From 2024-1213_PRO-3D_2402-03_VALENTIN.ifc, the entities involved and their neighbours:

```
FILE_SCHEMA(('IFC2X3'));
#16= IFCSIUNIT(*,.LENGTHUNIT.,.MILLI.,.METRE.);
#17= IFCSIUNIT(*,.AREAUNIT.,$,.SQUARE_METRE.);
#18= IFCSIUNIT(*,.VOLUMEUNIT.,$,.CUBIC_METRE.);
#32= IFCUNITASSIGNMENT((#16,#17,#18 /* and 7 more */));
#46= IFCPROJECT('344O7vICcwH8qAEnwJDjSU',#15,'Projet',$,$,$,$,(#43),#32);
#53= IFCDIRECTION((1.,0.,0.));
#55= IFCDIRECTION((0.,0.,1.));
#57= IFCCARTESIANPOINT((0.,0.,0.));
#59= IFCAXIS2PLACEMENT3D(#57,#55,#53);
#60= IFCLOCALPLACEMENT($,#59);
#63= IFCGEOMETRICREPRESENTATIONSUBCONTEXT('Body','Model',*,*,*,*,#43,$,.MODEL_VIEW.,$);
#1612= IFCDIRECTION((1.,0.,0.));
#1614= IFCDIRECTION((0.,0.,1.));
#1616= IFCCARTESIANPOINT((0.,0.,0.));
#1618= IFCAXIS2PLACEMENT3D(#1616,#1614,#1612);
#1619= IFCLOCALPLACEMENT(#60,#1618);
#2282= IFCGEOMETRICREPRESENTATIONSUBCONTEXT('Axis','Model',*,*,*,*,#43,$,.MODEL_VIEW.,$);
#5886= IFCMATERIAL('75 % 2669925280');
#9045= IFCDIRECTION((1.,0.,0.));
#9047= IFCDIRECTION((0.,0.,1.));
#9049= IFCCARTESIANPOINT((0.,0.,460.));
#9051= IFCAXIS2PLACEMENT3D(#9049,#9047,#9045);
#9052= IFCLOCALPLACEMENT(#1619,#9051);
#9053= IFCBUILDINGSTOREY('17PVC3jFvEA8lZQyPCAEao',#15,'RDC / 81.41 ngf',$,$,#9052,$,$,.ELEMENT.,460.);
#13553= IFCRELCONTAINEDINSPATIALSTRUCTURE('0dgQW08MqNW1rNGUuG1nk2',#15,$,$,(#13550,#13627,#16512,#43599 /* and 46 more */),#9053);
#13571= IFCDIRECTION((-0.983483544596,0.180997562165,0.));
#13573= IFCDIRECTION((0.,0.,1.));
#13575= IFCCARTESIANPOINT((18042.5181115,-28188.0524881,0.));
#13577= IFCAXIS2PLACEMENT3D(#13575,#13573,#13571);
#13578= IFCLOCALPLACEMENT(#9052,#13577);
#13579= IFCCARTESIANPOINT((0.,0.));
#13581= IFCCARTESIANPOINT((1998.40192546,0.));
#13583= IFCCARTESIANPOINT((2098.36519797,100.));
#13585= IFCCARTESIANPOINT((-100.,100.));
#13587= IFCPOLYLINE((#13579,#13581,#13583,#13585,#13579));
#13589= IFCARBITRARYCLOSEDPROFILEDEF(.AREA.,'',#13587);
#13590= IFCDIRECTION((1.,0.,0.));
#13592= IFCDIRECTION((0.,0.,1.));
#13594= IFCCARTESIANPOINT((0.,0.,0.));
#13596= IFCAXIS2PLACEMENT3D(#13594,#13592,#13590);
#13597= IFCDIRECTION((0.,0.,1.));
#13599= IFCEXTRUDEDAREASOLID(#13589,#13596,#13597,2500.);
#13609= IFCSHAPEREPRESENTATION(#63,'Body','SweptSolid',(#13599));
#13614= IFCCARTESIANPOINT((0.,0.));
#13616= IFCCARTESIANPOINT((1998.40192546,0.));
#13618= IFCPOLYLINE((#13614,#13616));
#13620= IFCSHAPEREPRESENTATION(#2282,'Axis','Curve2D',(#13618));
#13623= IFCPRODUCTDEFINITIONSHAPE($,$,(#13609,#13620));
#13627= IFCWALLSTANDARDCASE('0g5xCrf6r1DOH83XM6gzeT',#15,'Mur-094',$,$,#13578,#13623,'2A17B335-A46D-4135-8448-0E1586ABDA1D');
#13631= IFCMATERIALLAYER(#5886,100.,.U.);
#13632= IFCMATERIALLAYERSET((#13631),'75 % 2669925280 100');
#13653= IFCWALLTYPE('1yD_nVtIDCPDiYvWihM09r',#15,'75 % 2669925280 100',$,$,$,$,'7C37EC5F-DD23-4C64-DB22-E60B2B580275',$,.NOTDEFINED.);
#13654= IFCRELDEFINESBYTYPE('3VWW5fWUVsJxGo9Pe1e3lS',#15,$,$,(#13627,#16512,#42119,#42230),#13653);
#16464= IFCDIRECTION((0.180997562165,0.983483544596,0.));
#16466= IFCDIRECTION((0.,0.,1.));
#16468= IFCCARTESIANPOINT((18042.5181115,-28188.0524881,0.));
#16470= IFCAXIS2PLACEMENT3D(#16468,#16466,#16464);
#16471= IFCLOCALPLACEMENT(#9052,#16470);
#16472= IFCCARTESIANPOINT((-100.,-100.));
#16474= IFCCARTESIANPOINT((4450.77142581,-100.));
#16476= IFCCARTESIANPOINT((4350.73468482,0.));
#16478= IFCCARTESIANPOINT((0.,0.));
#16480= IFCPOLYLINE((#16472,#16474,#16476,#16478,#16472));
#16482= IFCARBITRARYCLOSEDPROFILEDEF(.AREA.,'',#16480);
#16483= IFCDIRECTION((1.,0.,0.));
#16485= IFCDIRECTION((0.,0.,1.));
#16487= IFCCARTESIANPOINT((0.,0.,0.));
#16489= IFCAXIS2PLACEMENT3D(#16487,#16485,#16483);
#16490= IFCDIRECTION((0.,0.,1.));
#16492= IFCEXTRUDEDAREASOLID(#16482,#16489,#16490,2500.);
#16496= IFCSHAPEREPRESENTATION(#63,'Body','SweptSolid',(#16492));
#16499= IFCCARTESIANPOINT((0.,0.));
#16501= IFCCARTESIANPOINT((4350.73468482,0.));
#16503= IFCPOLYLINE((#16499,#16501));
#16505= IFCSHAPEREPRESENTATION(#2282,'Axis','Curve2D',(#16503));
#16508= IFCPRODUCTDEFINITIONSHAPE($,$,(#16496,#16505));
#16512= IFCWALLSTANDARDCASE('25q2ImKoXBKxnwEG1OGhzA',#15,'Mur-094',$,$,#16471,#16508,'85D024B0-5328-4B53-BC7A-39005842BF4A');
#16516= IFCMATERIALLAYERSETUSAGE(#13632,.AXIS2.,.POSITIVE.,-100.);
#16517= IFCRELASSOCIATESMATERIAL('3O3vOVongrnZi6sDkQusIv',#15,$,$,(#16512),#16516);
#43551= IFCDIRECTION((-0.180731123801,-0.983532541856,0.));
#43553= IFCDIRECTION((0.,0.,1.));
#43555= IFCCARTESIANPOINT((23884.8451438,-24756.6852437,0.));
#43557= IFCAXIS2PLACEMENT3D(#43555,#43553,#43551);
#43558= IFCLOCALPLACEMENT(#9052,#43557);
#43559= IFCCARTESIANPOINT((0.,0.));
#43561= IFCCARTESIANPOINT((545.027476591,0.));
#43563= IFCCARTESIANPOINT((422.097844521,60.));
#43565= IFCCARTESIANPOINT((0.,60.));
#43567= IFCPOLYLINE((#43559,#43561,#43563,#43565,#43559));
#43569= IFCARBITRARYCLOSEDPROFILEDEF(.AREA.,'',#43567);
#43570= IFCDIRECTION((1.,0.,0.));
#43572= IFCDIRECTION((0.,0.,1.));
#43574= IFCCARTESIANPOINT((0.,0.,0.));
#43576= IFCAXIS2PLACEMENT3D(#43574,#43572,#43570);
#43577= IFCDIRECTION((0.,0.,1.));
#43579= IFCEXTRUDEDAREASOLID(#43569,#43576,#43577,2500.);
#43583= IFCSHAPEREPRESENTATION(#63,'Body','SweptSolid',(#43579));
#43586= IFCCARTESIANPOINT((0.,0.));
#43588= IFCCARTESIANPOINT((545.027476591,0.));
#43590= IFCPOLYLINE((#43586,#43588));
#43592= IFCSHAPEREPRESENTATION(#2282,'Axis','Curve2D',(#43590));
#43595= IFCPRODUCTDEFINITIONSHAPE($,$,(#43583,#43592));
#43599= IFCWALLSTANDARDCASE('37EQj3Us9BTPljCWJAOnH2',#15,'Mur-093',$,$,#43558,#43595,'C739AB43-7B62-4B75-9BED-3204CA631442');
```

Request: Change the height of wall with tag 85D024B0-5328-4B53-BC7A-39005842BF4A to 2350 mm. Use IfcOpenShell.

```python
import ifcopenshell
import ifcopenshell.geom
import ifcopenshell.util.representation
import ifcopenshell.util.shape

model = ifcopenshell.open("2024-1213_PRO-3D_2402-03_VALENTIN.ifc")
settings = ifcopenshell.geom.settings()


def volume(element):
    """Net volume in cubic metres, openings subtracted."""
    shape = ifcopenshell.geom.create_shape(settings, element)
    return ifcopenshell.util.shape.get_volume(shape.geometry)


wall = model.by_guid("25q2ImKoXBKxnwEG1OGhzA")
before = volume(wall)

body = ifcopenshell.util.representation.get_representation(wall, "Model", "Body")
solid = body.Items[0]
old_height = solid.Depth
solid.Depth = 2350.0
after = volume(wall)

print(f"height {old_height:g} -> {solid.Depth:g}, volume {before:.3f} -> {after:.3f} m3")

model.write("2024-1213_PRO-3D_2402-03_VALENTIN_updated.ifc")
```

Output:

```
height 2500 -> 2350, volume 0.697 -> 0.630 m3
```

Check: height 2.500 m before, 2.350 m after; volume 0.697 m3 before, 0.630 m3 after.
